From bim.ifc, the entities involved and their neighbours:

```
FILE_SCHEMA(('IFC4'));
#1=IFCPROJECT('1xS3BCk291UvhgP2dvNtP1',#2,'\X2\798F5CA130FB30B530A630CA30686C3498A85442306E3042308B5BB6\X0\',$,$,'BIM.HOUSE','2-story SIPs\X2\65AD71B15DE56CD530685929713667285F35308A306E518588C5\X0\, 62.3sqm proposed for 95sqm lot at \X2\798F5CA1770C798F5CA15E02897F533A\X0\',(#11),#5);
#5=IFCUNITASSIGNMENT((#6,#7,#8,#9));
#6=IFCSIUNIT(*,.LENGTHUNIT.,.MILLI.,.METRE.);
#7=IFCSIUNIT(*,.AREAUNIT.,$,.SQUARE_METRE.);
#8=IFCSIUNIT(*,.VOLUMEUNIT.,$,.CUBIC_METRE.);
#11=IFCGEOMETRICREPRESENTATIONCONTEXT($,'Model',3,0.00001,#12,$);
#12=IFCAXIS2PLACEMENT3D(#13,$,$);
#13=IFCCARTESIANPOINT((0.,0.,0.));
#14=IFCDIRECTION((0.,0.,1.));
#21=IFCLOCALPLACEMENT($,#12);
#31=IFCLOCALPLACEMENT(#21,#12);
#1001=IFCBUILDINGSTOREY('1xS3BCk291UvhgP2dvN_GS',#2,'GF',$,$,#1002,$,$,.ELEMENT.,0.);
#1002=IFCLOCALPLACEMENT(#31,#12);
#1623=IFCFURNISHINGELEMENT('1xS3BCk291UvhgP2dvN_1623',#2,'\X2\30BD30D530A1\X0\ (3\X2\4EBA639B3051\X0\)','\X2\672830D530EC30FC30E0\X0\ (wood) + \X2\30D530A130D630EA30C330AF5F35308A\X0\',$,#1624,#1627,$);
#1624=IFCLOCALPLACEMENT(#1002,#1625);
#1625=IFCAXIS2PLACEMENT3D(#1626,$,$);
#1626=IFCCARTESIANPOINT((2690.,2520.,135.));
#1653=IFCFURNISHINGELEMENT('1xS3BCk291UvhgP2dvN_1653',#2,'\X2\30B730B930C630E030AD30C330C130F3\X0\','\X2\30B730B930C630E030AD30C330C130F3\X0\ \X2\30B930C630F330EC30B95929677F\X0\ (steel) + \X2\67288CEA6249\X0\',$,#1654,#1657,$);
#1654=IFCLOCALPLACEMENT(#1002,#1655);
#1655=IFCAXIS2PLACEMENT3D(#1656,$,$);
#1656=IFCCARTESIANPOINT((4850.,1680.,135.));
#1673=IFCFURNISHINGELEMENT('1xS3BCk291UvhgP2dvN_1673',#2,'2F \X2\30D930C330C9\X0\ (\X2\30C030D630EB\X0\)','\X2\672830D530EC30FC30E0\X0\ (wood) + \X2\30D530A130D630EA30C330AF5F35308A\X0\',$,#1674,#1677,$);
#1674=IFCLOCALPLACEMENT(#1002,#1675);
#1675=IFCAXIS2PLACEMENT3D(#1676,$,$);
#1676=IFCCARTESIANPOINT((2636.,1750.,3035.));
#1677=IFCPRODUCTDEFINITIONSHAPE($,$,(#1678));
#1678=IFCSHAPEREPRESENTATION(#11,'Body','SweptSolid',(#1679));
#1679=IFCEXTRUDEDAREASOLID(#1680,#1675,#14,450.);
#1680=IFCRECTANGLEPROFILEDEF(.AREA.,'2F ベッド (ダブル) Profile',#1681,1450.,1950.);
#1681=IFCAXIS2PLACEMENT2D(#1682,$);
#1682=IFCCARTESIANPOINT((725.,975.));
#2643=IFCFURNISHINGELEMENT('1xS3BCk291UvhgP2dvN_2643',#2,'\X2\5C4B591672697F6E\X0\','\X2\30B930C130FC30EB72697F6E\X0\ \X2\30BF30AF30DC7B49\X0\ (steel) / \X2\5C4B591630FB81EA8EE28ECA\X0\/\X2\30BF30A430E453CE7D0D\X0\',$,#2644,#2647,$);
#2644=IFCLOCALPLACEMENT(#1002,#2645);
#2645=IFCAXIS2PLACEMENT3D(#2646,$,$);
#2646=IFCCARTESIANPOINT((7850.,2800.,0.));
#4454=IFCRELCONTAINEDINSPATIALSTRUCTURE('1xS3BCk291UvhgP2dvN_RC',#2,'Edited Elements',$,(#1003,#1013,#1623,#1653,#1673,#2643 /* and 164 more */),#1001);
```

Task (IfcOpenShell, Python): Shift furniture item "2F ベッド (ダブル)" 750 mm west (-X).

```python
import ifcopenshell
import ifcopenshell.api.geometry
import ifcopenshell.util.placement

model = ifcopenshell.open("bim.ifc")

item = model.by_guid("1xS3BCk291UvhgP2dvN_1673")
matrix = ifcopenshell.util.placement.get_local_placement(item.ObjectPlacement)
matrix[0, 3] -= 750.0
ifcopenshell.api.geometry.edit_object_placement(model, product=item, matrix=matrix, is_si=False)

print(ifcopenshell.util.placement.get_local_placement(item.ObjectPlacement).round(3) + 0.0)

model.write("bim_rev.ifc")
```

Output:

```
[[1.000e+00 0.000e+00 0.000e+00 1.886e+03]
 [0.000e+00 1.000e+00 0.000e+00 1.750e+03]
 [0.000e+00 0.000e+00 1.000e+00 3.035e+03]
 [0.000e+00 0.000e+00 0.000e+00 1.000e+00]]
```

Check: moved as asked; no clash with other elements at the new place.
